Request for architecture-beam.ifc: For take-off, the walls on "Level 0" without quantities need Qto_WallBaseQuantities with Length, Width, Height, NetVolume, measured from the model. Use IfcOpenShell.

First a look at what the model holds.

```python
import ifcopenshell
import ifcopenshell.util.element
import ifcopenshell.util.unit

model = ifcopenshell.open("architecture-beam.ifc")
print(model.schema)
for unit_type in ("LENGTHUNIT", "AREAUNIT", "VOLUMEUNIT"):
    print(unit_type, ifcopenshell.util.unit.calculate_unit_scale(model, unit_type))
storey = next(s for s in model.by_type("IfcBuildingStorey") if s.Name == "Level 0")
walls = [e for e in ifcopenshell.util.element.get_decomposition(storey) if e.is_a("IfcWall")]
for e in sorted(walls, key=lambda e: e.id()):
    print(e.id(), e.is_a(), e.Name, list(ifcopenshell.util.element.get_psets(e, qtos_only=True)), sep=" | ")
```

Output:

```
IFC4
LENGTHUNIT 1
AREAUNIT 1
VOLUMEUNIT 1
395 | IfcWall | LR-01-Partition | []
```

```python
import ifcopenshell
import ifcopenshell.api.pset
import ifcopenshell.geom
import ifcopenshell.util.element
import ifcopenshell.util.shape
import ifcopenshell.util.unit

model = ifcopenshell.open("architecture-beam.ifc")
unit_scale = ifcopenshell.util.unit.calculate_unit_scale(model)
volume_scale = ifcopenshell.util.unit.calculate_unit_scale(model, "VOLUMEUNIT")
settings = ifcopenshell.geom.settings()

storey = next(s for s in model.by_type("IfcBuildingStorey") if s.Name == "Level 0")
walls = [e for e in ifcopenshell.util.element.get_decomposition(storey) if e.is_a("IfcWall")]

for e in sorted(walls, key=lambda e: e.id()):
    if ifcopenshell.util.element.get_psets(e, qtos_only=True, should_inherit=False):
        continue
    # Geometry comes back in metres, in the element's own axes.
    shape = ifcopenshell.geom.create_shape(settings, e)
    values = {
        "Length": ifcopenshell.util.shape.get_x(shape.geometry) / unit_scale,
        "Width": ifcopenshell.util.shape.get_y(shape.geometry) / unit_scale,
        "Height": ifcopenshell.util.shape.get_z(shape.geometry) / unit_scale,
        "NetVolume": ifcopenshell.util.shape.get_volume(shape.geometry) / volume_scale,
    }
    qto = ifcopenshell.api.pset.add_qto(model, product=e, name="Qto_WallBaseQuantities")
    ifcopenshell.api.pset.edit_qto(model, qto=qto, properties=values)
    print(e.id(), {k: round(v, 3) for k, v in values.items()})

model.write("architecture-beam_v2.ifc")
```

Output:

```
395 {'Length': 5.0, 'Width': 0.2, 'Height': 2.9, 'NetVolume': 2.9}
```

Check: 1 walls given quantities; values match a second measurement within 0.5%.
